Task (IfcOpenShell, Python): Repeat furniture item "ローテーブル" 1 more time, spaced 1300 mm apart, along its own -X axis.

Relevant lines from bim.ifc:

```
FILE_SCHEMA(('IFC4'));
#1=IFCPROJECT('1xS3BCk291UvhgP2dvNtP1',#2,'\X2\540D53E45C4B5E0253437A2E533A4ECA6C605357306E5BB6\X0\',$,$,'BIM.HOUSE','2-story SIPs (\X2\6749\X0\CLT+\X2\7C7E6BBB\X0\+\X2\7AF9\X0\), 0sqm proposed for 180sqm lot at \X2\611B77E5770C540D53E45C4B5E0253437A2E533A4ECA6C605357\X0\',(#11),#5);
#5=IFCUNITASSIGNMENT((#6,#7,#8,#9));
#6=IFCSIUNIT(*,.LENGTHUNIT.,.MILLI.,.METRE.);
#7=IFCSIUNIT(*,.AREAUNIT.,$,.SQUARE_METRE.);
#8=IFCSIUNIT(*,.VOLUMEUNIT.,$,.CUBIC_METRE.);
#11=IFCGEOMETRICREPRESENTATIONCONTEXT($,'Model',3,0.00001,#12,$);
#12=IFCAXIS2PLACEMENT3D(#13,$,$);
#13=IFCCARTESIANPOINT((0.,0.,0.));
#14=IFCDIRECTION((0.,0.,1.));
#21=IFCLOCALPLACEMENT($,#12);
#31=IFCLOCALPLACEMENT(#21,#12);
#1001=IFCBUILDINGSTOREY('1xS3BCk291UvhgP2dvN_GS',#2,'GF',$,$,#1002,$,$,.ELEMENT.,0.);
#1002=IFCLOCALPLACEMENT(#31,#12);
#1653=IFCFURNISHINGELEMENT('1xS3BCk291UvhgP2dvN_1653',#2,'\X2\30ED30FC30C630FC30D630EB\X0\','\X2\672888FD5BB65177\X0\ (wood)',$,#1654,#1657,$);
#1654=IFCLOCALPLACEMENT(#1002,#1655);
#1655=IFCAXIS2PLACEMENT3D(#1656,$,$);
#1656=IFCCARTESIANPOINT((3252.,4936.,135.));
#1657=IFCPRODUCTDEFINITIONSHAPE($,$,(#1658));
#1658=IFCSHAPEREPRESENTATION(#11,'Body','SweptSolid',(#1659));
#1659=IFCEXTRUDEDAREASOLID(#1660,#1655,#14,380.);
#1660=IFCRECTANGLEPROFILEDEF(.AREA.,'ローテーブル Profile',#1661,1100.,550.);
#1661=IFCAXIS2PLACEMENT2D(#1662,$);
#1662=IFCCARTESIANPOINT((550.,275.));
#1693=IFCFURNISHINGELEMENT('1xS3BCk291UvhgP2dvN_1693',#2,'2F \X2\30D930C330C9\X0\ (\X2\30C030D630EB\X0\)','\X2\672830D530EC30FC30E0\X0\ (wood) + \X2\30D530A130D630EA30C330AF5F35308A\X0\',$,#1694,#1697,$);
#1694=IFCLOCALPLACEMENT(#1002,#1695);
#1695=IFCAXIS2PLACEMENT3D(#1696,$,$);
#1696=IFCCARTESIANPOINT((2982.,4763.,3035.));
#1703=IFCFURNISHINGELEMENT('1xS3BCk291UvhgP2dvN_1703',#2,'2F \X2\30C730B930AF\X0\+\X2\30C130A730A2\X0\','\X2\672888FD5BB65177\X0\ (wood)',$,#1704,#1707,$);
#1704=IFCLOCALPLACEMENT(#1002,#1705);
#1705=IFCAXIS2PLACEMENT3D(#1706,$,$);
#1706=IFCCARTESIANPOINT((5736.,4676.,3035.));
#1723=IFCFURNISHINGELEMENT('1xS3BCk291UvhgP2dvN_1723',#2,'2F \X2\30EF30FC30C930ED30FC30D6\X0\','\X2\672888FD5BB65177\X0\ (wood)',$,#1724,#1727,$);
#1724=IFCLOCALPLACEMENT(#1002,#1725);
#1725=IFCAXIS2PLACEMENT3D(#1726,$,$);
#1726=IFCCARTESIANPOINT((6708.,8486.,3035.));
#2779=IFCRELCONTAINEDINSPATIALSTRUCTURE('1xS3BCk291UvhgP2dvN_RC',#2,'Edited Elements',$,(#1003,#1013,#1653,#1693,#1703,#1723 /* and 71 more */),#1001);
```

```python
import ifcopenshell
import ifcopenshell.api.geometry
import ifcopenshell.api.root
import ifcopenshell.util.element
import ifcopenshell.util.placement
import ifcopenshell.util.unit

model = ifcopenshell.open("bim.ifc")
unit_scale = ifcopenshell.util.unit.calculate_unit_scale(model)


def reuse_history(source, copy):
    """copy_class also copies each property set's owner history, people and application; keep the originals."""
    for rel in copy.IsDefinedBy:
        if rel.is_a("IfcRelDefinesByProperties") and (history := rel.RelatingPropertyDefinition.OwnerHistory):
            rel.RelatingPropertyDefinition.OwnerHistory = source.OwnerHistory
            ifcopenshell.util.element.remove_deep2(model, history)


source = model.by_guid("1xS3BCk291UvhgP2dvN_1653")
base = ifcopenshell.util.placement.get_local_placement(source.ObjectPlacement)
step = -base[:3, 0] * 1.3 / unit_scale

for i in range(1, 2):
    copy = ifcopenshell.api.root.copy_class(model, product=source)
    copy.Representation = ifcopenshell.util.element.copy_deep(
        model, source.Representation, exclude=["IfcGeometricRepresentationContext", "IfcRepresentationMap"]
    )
    reuse_history(source, copy)
    matrix = base.copy()
    matrix[:3, 3] += i * step
    print("added at", matrix[:3, 3].round(3) + 0.0)
    ifcopenshell.api.geometry.edit_object_placement(model, product=copy, matrix=matrix, is_si=False)

model.write("bim_v2.ifc")
```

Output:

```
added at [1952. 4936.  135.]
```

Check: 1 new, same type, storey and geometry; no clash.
